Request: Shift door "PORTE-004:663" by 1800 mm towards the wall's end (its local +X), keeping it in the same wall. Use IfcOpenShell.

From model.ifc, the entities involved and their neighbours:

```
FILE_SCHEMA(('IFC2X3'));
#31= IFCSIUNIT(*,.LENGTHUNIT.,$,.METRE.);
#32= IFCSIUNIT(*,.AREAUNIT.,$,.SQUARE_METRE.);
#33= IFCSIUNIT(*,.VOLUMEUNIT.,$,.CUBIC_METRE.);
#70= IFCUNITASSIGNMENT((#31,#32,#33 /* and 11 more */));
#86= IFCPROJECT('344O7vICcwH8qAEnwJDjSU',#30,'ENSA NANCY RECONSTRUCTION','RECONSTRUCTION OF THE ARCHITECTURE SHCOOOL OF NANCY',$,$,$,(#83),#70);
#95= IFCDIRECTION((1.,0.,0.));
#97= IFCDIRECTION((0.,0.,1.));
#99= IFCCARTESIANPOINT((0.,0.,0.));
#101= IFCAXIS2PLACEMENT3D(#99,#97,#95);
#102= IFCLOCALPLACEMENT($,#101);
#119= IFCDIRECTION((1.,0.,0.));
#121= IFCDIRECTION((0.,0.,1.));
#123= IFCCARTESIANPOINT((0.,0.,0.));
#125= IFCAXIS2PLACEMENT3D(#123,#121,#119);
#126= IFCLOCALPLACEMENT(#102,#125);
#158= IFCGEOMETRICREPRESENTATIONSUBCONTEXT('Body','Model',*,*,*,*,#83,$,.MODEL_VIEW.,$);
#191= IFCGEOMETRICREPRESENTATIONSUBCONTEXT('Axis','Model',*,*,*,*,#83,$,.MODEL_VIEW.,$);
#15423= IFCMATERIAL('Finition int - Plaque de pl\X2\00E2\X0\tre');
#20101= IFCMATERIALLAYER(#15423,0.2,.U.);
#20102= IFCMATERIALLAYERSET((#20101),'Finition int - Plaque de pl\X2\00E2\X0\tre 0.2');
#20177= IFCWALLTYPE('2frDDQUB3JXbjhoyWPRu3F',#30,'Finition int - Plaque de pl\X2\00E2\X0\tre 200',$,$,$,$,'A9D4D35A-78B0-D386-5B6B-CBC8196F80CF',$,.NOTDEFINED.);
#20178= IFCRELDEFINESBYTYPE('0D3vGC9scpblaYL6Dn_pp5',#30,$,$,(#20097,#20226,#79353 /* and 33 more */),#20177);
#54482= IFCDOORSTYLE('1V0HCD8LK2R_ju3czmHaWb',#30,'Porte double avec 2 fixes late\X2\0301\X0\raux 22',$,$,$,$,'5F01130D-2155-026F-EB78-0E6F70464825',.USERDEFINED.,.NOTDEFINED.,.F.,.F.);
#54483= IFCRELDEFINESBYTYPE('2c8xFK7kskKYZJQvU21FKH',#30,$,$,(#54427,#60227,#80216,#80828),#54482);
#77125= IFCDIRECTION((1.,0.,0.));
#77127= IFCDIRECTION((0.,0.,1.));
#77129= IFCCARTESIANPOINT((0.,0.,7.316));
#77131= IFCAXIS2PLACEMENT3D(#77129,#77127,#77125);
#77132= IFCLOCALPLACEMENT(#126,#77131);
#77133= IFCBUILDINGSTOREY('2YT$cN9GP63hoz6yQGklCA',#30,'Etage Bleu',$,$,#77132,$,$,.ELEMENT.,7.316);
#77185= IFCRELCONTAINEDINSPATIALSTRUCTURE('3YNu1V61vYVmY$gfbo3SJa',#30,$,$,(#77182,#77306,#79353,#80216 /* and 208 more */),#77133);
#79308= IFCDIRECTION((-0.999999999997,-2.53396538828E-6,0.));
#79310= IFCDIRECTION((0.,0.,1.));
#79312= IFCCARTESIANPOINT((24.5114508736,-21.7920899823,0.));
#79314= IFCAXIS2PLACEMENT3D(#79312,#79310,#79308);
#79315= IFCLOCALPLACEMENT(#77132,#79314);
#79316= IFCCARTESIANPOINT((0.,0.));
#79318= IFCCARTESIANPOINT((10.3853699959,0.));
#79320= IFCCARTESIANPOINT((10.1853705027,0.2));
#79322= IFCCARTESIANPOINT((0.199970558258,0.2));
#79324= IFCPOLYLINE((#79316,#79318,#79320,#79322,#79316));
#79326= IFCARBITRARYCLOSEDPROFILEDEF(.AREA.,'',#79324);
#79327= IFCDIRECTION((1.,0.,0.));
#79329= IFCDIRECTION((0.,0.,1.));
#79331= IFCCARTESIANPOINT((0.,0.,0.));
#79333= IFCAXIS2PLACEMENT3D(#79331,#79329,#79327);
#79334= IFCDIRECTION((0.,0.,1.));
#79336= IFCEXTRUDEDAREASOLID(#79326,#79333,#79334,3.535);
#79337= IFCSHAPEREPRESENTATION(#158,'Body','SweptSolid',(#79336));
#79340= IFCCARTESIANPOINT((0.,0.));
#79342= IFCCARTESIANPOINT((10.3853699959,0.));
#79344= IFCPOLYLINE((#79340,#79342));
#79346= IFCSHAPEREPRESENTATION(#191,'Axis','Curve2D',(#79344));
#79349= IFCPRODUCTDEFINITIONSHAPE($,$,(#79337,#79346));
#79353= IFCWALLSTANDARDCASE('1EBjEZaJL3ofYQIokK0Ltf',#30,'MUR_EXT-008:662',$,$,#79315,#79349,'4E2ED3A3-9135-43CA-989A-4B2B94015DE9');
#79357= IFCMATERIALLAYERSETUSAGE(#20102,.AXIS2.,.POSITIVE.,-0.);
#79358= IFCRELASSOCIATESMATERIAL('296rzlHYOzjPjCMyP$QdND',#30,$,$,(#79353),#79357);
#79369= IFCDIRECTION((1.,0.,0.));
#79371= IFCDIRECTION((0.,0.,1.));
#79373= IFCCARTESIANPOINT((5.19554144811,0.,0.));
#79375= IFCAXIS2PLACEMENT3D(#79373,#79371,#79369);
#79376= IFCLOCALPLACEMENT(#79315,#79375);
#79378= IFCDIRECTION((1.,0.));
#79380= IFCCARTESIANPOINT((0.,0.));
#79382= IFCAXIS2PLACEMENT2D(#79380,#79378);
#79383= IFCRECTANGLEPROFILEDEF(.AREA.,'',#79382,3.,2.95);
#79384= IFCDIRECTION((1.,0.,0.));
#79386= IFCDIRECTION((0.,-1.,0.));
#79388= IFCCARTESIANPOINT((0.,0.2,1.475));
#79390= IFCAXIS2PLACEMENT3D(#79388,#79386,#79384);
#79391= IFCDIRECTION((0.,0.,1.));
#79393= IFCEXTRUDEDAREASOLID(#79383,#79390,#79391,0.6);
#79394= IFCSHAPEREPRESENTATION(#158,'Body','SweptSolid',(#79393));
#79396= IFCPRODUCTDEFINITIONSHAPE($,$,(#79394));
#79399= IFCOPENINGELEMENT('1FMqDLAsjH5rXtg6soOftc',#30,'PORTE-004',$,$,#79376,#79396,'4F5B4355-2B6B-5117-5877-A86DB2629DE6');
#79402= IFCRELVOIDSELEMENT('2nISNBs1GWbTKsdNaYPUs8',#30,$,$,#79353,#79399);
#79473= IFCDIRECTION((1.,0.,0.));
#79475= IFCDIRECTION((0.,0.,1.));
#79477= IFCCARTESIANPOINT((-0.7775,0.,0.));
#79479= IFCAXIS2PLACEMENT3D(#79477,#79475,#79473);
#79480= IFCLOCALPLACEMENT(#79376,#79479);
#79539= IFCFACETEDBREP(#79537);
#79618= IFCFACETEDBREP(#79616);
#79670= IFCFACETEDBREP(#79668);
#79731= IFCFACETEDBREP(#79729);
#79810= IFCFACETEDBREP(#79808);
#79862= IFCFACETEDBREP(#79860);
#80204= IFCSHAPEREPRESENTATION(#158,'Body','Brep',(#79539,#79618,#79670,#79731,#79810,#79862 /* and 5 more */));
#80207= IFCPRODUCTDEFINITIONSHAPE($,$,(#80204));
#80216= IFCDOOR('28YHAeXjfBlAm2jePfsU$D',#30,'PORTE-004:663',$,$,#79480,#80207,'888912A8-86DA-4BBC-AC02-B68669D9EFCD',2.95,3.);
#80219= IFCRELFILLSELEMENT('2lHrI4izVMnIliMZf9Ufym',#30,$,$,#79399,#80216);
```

```python
import ifcopenshell
import ifcopenshell.api.geometry
import ifcopenshell.util.placement

model = ifcopenshell.open("model.ifc")

door = model.by_guid("28YHAeXjfBlAm2jePfsU$D")
opening = door.FillsVoids[0].RelatingOpeningElement
wall = opening.VoidsElements[0].RelatingBuildingElement

wall_matrix = ifcopenshell.util.placement.get_local_placement(wall.ObjectPlacement)
shift = wall_matrix[:3, 0] * 1.8
before = ifcopenshell.util.placement.get_local_placement(door.ObjectPlacement)[:3, 3].copy()

# The door is placed relative to its opening, so it follows when the opening moves.
matrix = ifcopenshell.util.placement.get_local_placement(opening.ObjectPlacement)
matrix[:3, 3] += shift
ifcopenshell.api.geometry.edit_object_placement(
    model, product=opening, matrix=matrix, is_si=False, should_transform_children=True
)

after = ifcopenshell.util.placement.get_local_placement(door.ObjectPlacement)[:3, 3]
print("door moved by", (after - before).round(3) + 0.0)

model.write("model_edited.ifc")
```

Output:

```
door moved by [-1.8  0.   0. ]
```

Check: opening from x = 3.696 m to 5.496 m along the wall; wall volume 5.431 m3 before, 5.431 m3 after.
